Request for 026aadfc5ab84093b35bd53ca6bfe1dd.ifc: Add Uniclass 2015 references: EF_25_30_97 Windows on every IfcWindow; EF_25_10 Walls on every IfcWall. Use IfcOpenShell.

First a look at what the model holds.

```python
import ifcopenshell

model = ifcopenshell.open("026aadfc5ab84093b35bd53ca6bfe1dd.ifc")
print(model.schema)
print("classifications:", [c.Name for c in model.by_type("IfcClassification")])
for ifc_class in ("IfcDoor", "IfcRoof", "IfcStair", "IfcWall", "IfcWindow"):
    print(ifc_class, len(model.by_type(ifc_class)))
```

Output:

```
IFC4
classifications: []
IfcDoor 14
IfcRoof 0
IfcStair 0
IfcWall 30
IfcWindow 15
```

```python
import ifcopenshell
import ifcopenshell.api.classification

model = ifcopenshell.open("026aadfc5ab84093b35bd53ca6bfe1dd.ifc")

system = ifcopenshell.api.classification.add_classification(model, classification="Uniclass 2015")

codes = {
    "IfcWindow": ("EF_25_30_97", "Windows"),
    "IfcWall": ("EF_25_10", "Walls"),
}
for ifc_class, (code, name) in codes.items():
    products = model.by_type(ifc_class)
    ifcopenshell.api.classification.add_reference(
        model, products=products, classification=system, identification=code, name=name
    )
    print(code, len(products))

model.write("026aadfc5ab84093b35bd53ca6bfe1dd_v2.ifc")
```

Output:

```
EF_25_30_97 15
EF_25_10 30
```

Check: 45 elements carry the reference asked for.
